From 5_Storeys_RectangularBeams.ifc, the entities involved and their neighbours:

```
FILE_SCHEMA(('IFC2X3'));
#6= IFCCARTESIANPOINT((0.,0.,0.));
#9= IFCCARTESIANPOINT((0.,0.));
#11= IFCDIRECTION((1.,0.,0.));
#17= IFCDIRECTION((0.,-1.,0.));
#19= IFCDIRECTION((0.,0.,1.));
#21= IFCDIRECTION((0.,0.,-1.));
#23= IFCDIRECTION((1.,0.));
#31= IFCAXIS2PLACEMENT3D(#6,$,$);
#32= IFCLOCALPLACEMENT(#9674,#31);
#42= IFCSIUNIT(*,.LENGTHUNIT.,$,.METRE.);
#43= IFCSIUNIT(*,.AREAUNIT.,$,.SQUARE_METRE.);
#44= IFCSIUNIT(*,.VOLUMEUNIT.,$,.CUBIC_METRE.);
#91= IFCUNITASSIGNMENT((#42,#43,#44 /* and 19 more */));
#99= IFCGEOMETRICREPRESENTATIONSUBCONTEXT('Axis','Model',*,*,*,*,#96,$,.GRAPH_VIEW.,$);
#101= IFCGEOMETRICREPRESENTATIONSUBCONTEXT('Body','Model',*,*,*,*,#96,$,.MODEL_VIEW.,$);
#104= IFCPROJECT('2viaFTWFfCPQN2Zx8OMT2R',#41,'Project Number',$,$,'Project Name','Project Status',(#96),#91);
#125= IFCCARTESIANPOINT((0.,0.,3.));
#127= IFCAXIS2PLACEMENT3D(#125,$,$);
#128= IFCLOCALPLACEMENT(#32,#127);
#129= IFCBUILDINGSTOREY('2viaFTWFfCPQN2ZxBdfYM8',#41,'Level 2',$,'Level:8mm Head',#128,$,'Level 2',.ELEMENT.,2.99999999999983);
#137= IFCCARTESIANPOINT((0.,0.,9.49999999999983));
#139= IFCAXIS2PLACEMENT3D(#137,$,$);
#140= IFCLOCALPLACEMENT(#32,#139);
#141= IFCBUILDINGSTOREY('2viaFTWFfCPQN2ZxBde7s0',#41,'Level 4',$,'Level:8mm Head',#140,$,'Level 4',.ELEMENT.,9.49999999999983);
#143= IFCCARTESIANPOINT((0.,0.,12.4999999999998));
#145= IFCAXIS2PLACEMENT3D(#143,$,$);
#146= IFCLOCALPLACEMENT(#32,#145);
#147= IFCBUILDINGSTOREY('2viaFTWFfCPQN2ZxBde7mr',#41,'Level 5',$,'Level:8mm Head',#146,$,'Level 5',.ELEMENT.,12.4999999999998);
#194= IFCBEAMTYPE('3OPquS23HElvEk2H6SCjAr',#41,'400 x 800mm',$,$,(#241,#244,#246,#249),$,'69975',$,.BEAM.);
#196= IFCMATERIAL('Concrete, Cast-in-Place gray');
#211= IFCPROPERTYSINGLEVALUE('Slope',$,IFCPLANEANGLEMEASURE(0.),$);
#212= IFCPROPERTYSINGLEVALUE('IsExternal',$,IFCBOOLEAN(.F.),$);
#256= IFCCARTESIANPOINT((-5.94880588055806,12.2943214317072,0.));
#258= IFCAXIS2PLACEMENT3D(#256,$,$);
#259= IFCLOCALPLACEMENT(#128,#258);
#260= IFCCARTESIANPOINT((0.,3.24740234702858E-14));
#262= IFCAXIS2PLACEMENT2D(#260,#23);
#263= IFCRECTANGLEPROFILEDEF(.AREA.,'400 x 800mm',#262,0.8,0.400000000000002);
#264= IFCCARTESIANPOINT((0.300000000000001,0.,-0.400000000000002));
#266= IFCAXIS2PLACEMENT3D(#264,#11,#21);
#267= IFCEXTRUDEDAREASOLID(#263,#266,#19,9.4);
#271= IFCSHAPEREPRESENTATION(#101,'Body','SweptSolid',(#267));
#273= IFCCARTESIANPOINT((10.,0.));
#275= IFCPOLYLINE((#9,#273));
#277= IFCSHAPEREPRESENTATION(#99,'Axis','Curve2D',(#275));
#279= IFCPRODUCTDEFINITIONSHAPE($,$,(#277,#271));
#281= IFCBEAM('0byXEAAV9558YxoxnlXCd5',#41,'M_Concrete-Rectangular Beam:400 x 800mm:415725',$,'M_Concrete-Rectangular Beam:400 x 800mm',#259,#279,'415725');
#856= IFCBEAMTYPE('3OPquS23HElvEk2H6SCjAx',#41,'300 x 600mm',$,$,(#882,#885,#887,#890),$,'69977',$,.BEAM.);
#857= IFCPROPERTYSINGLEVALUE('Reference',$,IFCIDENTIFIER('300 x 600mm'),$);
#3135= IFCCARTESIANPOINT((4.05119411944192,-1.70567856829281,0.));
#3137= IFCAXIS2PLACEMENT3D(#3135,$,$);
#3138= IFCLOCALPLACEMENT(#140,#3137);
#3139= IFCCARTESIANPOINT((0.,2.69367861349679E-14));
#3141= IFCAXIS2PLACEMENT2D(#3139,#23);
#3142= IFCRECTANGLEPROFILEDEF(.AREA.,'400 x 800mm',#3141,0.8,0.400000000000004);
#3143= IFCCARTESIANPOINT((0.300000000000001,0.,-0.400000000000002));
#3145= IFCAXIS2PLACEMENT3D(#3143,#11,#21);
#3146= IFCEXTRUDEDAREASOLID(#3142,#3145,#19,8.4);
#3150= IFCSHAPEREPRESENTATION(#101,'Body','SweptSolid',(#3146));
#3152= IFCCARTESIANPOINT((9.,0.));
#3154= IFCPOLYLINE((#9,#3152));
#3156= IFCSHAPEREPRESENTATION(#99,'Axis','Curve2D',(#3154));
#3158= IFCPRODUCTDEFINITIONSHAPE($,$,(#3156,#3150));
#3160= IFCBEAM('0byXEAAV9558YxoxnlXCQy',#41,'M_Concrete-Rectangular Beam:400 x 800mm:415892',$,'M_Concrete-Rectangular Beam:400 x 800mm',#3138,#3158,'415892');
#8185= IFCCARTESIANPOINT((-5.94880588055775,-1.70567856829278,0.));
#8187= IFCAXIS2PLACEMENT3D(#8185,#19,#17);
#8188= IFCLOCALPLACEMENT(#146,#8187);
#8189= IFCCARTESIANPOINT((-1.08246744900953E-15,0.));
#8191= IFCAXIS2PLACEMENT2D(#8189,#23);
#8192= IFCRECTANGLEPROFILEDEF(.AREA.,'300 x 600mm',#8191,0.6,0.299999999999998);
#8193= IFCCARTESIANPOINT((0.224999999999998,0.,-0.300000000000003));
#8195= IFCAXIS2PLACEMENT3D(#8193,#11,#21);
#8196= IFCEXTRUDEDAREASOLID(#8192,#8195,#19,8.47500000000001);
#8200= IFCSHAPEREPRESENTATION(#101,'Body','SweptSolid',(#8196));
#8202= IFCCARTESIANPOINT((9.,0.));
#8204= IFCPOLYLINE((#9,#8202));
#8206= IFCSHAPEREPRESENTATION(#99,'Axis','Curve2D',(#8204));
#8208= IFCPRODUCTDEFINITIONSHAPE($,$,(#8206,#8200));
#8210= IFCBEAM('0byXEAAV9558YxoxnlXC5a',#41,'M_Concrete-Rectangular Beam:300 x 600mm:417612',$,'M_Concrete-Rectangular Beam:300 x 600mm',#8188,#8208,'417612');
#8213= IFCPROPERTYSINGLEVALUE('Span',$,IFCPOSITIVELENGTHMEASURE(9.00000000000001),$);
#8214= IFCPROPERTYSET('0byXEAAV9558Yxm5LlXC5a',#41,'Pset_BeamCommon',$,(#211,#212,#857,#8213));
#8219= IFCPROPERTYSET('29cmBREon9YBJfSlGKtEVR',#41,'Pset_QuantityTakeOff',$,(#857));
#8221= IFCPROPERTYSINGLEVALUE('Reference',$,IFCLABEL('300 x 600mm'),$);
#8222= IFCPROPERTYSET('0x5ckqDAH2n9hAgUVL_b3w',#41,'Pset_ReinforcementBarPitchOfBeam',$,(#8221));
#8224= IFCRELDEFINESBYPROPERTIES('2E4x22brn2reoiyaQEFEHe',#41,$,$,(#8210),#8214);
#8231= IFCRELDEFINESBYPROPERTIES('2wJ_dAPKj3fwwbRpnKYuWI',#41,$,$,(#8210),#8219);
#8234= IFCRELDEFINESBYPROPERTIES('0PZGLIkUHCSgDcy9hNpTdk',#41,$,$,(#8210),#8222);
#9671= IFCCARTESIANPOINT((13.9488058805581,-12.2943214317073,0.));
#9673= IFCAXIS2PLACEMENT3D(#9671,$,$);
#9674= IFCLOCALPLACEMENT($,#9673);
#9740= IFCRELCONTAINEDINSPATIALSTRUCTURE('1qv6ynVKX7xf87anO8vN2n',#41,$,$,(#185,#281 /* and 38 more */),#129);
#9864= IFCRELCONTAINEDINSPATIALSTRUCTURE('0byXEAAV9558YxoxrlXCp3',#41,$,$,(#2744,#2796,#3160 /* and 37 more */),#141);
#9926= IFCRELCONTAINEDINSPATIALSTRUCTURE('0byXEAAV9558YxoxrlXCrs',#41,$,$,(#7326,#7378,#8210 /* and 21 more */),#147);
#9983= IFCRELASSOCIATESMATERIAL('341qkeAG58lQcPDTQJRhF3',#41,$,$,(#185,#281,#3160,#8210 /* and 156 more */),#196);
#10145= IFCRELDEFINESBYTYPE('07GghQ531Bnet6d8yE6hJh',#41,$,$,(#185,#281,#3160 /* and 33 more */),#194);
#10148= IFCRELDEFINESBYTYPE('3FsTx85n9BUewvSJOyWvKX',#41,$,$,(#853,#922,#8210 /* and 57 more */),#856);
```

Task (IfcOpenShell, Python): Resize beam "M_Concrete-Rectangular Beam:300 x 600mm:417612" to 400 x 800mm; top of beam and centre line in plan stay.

```python
import ifcopenshell
import ifcopenshell.api.pset
import ifcopenshell.api.type
import ifcopenshell.util.element
import ifcopenshell.util.representation

model = ifcopenshell.open("5_Storeys_RectangularBeams.ifc")

member = model.by_guid("0byXEAAV9558YxoxnlXC5a")
source = next(p for p in model.by_type("IfcRectangleProfileDef") if p.ProfileName == "400 x 800mm")

body = ifcopenshell.util.representation.get_representation(member, "Model", "Body")
solid = body.Items[0]
old_profile = solid.SweptArea

# Copy the section's sizes but keep this member's own profile position.
profile = ifcopenshell.util.element.copy(model, source)
# Profiles are centred, so shift by half the change in depth to hold the top.
shift = (old_profile.XDim - profile.XDim) / 2
x, y = old_profile.Position.Location.Coordinates
up = (-1.0, 0.0)  # upwards, in the solid's own plane
location = model.createIfcCartesianPoint((x + up[0] * shift, y + up[1] * shift))
profile.Position = model.createIfcAxis2Placement2D(location, old_profile.Position.RefDirection)
solid.SweptArea = profile
if not model.get_total_inverses(old_profile):
    ifcopenshell.util.element.remove_deep2(model, old_profile)

new_type = model.by_guid("3OPquS23HElvEk2H6SCjAr")
ifcopenshell.api.type.assign_type(
    model, related_objects=[member], relating_type=new_type, should_map_representations=False
)
member.Name = member.Name.replace("300 x 600mm", "400 x 800mm")
member.ObjectType = "M_Concrete-Rectangular Beam:400 x 800mm"
pset = model.by_id(ifcopenshell.util.element.get_pset(member, "Pset_BeamCommon", should_inherit=False)["id"])
ifcopenshell.api.pset.edit_pset(model, pset=pset, properties={"Reference": "400 x 800mm"})
pset = model.by_id(ifcopenshell.util.element.get_pset(member, "Pset_QuantityTakeOff", should_inherit=False)["id"])
ifcopenshell.api.pset.edit_pset(model, pset=pset, properties={"Reference": "400 x 800mm"})
pset = model.by_id(ifcopenshell.util.element.get_pset(member, "Pset_ReinforcementBarPitchOfBeam", should_inherit=False)["id"])
ifcopenshell.api.pset.edit_pset(model, pset=pset, properties={"Reference": "400 x 800mm"})

print(solid.SweptArea)

model.write("5_Storeys_RectangularBeams_updated.ifc")
```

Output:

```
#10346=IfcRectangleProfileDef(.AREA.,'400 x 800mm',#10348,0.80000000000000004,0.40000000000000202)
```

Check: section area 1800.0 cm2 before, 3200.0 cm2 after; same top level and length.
